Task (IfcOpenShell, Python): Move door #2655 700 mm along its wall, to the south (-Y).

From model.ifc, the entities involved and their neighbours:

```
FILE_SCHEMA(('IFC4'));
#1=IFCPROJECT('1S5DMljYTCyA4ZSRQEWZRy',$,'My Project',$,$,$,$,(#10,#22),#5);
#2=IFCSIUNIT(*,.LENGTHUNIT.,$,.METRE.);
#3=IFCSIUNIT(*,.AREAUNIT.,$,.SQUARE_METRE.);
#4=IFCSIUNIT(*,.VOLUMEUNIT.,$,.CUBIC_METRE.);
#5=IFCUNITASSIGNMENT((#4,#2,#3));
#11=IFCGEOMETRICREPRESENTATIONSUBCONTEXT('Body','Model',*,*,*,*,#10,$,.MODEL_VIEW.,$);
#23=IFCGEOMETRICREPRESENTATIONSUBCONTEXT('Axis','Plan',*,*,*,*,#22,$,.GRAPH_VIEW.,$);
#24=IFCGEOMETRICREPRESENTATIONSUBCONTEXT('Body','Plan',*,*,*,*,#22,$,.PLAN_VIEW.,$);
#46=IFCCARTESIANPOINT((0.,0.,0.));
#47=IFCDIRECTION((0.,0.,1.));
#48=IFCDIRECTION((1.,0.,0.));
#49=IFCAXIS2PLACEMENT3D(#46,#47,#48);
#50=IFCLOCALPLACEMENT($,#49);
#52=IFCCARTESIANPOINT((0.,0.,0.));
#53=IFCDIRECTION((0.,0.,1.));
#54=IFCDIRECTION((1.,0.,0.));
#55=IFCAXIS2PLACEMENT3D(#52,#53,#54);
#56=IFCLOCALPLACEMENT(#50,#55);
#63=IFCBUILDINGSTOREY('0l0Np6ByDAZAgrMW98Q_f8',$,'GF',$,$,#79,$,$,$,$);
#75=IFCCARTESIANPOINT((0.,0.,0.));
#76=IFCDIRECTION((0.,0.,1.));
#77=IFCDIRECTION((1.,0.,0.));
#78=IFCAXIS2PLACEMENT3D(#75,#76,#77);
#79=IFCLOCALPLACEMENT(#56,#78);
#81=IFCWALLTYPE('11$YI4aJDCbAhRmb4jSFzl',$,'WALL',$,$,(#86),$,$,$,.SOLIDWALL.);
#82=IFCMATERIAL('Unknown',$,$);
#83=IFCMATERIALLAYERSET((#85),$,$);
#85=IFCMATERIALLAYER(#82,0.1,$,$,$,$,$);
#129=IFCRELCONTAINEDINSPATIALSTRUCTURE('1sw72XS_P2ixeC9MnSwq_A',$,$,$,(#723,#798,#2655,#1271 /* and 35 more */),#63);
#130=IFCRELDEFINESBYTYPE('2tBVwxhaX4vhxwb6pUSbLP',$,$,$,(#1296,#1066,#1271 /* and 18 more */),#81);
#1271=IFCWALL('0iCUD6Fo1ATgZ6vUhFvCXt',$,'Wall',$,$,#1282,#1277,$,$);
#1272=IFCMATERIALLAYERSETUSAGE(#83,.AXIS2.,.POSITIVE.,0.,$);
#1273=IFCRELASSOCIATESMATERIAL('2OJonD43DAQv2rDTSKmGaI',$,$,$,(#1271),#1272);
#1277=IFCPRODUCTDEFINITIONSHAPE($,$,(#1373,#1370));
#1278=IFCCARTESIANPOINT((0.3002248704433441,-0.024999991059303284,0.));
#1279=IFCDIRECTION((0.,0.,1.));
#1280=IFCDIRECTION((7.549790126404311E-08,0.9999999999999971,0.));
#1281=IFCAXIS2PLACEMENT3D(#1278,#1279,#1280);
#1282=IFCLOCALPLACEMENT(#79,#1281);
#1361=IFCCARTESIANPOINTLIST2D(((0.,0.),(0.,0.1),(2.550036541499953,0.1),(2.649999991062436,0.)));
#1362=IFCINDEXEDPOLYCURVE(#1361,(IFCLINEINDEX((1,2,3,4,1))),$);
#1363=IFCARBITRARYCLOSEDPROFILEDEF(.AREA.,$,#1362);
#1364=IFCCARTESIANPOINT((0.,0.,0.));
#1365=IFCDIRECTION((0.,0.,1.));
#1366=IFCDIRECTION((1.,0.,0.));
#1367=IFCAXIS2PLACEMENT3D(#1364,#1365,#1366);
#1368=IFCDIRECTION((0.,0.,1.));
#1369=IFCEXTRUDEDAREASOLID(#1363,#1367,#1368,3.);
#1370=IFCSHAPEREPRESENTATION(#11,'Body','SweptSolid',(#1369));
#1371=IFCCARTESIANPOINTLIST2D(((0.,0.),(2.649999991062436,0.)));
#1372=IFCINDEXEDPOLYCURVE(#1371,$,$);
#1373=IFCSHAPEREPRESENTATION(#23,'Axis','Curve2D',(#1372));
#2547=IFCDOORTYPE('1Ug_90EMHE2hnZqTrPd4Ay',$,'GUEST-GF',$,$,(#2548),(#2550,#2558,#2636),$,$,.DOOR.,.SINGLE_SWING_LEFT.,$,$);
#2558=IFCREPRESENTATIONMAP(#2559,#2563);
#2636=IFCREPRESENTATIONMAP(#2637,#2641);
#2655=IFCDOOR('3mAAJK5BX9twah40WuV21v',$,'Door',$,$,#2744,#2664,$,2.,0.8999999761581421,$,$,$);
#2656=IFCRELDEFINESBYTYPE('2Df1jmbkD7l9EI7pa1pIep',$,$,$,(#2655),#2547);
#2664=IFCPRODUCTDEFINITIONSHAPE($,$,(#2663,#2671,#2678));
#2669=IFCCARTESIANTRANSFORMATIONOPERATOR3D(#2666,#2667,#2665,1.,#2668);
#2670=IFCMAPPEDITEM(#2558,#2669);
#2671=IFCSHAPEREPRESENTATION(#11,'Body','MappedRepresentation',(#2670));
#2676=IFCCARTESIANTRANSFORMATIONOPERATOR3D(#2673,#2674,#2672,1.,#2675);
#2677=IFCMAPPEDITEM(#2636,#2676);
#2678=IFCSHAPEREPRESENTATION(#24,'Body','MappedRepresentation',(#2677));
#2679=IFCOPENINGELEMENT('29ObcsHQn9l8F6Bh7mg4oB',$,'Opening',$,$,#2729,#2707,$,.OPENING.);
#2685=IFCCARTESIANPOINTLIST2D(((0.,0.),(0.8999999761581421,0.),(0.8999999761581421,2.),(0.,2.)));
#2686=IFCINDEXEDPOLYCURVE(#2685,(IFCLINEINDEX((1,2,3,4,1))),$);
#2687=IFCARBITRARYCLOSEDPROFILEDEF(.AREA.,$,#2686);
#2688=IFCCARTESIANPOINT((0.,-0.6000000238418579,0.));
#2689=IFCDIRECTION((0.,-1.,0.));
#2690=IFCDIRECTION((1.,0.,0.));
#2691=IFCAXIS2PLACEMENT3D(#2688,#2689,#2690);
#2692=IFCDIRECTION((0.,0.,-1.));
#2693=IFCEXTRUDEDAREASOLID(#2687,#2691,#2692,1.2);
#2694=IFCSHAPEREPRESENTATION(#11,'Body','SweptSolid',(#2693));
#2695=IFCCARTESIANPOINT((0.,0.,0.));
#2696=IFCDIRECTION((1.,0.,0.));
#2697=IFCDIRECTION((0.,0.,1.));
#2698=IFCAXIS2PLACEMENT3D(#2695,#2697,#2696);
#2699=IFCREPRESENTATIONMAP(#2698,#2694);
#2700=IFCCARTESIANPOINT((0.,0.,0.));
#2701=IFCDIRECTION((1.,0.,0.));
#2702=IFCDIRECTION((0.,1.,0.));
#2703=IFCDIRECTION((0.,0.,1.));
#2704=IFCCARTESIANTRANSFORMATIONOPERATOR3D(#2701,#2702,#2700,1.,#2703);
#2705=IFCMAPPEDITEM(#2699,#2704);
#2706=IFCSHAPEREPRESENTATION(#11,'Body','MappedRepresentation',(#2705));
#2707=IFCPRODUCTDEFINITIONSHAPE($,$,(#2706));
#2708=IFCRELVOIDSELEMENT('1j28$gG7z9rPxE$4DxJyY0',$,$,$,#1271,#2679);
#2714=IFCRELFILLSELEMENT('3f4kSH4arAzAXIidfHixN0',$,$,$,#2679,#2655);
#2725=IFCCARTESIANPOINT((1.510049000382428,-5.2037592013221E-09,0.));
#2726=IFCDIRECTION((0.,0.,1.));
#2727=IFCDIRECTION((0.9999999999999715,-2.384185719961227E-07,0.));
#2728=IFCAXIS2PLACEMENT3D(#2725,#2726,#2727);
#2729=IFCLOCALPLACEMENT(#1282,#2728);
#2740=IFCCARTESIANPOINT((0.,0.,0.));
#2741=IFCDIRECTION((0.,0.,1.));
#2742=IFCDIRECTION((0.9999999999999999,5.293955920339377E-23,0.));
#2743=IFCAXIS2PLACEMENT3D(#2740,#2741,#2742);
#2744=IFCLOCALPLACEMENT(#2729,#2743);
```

```python
import ifcopenshell
import ifcopenshell.api.geometry
import ifcopenshell.util.placement
import ifcopenshell.util.unit

model = ifcopenshell.open("model.ifc")
unit_scale = ifcopenshell.util.unit.calculate_unit_scale(model)

door = model.by_id(2655)
opening = door.FillsVoids[0].RelatingOpeningElement
wall = opening.VoidsElements[0].RelatingBuildingElement

wall_matrix = ifcopenshell.util.placement.get_local_placement(wall.ObjectPlacement)
shift = wall_matrix[:3, 0] * -0.7 / unit_scale
before = ifcopenshell.util.placement.get_local_placement(door.ObjectPlacement)[:3, 3].copy()

# The door is placed relative to its opening, so it follows when the opening moves.
matrix = ifcopenshell.util.placement.get_local_placement(opening.ObjectPlacement)
matrix[:3, 3] += shift
ifcopenshell.api.geometry.edit_object_placement(
    model, product=opening, matrix=matrix, is_si=False, should_transform_children=True
)

after = ifcopenshell.util.placement.get_local_placement(door.ObjectPlacement)[:3, 3]
print("door moved by", (after - before).round(3) + 0.0)

model.write("model_rev.ifc")
```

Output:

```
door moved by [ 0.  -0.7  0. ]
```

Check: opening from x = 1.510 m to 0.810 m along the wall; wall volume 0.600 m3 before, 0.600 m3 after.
